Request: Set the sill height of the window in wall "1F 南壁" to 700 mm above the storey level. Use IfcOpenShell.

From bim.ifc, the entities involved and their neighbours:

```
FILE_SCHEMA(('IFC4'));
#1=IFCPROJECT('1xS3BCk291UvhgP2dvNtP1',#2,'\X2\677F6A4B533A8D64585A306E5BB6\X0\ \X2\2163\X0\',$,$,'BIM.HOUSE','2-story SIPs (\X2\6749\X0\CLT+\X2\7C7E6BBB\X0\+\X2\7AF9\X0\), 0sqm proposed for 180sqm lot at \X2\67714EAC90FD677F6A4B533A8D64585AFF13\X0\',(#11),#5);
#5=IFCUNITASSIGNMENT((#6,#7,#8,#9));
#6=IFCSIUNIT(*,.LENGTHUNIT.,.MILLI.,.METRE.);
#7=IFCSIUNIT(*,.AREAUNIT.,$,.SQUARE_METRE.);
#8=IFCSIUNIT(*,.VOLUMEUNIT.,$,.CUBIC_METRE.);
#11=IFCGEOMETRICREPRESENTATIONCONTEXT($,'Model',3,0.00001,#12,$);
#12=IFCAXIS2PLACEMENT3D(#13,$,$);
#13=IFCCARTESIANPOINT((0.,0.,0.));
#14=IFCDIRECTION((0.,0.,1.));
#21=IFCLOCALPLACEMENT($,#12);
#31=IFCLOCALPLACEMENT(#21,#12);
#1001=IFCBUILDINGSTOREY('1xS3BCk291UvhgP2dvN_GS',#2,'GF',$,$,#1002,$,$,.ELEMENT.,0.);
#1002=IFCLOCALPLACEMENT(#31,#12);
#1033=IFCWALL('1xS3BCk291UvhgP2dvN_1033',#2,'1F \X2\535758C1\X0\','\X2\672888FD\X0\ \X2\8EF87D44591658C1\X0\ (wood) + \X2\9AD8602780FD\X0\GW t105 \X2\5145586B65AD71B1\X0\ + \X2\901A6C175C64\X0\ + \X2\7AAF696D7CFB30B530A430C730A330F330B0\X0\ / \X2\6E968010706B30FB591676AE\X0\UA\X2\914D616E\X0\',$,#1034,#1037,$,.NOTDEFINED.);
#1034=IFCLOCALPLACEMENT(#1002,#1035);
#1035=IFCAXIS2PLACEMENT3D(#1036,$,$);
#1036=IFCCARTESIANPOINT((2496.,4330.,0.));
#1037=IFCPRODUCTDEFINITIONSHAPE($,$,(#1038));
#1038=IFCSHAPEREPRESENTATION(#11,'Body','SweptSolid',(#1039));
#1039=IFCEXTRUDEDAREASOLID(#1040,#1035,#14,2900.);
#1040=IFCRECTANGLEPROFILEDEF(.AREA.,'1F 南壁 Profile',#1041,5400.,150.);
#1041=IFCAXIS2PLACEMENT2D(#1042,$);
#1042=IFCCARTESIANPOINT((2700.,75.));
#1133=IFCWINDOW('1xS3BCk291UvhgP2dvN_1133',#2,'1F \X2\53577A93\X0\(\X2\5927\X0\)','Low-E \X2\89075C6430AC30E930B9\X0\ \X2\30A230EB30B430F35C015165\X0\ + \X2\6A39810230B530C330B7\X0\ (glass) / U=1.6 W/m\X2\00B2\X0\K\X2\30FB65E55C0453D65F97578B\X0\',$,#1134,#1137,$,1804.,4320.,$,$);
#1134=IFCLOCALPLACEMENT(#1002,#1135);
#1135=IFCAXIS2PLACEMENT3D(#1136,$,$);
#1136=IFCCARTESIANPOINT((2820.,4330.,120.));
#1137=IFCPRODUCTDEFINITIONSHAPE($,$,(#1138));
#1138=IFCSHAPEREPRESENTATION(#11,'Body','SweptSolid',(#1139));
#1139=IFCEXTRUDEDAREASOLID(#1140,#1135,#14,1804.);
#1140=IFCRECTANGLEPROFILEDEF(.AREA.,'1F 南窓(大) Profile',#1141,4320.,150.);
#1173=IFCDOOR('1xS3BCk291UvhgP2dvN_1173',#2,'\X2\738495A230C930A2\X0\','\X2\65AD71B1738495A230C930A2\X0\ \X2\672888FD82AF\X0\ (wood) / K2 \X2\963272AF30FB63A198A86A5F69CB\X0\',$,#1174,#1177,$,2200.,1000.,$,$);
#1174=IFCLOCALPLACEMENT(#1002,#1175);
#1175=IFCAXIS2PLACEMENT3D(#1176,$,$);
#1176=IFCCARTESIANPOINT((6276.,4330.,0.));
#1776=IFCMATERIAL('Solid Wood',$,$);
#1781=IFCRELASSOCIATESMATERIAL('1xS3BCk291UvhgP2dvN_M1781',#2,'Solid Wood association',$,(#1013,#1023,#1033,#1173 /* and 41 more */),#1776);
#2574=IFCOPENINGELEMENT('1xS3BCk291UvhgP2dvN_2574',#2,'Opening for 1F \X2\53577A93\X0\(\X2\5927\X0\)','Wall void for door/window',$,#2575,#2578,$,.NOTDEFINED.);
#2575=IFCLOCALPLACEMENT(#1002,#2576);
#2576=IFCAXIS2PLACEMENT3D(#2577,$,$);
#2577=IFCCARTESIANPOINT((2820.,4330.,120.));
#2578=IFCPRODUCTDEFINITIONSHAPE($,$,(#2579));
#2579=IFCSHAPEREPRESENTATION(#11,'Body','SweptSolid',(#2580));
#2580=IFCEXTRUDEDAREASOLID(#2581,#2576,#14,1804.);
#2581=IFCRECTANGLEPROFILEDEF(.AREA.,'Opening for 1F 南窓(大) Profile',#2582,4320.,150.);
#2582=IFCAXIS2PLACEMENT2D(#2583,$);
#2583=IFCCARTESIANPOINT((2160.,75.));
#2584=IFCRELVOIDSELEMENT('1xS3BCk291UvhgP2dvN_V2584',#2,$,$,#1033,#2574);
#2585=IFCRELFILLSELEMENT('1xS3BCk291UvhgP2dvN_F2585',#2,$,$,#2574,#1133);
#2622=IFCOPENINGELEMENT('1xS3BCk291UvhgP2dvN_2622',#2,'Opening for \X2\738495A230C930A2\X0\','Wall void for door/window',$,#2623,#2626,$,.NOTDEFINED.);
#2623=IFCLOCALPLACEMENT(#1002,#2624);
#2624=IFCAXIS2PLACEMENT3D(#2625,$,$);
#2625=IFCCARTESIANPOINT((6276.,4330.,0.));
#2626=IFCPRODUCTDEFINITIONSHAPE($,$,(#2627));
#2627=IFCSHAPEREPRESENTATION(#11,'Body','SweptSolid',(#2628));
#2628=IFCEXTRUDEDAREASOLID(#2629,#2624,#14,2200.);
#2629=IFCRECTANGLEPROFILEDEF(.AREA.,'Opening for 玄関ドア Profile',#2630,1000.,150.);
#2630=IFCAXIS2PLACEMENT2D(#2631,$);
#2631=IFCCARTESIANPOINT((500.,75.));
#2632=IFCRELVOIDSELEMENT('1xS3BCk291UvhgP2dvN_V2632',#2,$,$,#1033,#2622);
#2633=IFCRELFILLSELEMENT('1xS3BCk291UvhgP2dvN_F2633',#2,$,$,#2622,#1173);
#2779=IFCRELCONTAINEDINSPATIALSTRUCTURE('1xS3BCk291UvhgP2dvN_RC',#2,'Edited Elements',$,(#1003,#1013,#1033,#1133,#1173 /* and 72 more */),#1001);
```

```python
import numpy as np
import ifcopenshell
import ifcopenshell.api.geometry
import ifcopenshell.geom
import ifcopenshell.util.element
import ifcopenshell.util.placement
import ifcopenshell.util.shape
import ifcopenshell.util.unit

model = ifcopenshell.open("bim.ifc")
unit_scale = ifcopenshell.util.unit.calculate_unit_scale(model)

window = model.by_guid("1xS3BCk291UvhgP2dvN_1133")
opening = window.FillsVoids[0].RelatingOpeningElement
storey = ifcopenshell.util.element.get_container(window, ifc_class="IfcBuildingStorey")
level = ifcopenshell.util.placement.get_local_placement(storey.ObjectPlacement)[2, 3]

# The opening's origin need not be at the sill, so measure its lowest point.
shape = ifcopenshell.geom.create_shape(ifcopenshell.geom.settings(), opening)
bottom = ifcopenshell.util.shape.get_shape_bottom_elevation(shape, shape.geometry) / unit_scale
dz = level + 0.7 / unit_scale - bottom

shift = np.array([0.0, 0.0, dz])
# The window is not placed relative to its opening, so move both.
for product in (opening, window):
    matrix = ifcopenshell.util.placement.get_local_placement(product.ObjectPlacement)
    matrix[:3, 3] += shift
    ifcopenshell.api.geometry.edit_object_placement(model, product=product, matrix=matrix, is_si=False)

print(f"moved by {dz * unit_scale:+.3f} m")

model.write("bim_v2.ifc")
```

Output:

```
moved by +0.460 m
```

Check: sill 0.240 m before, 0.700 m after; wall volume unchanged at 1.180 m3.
